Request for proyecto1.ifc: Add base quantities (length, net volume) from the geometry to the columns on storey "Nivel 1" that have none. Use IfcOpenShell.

First a look at what the model holds.

```python
import ifcopenshell
import ifcopenshell.util.element
import ifcopenshell.util.unit

model = ifcopenshell.open("proyecto1.ifc")
print(model.schema)
for unit_type in ("LENGTHUNIT", "AREAUNIT", "VOLUMEUNIT"):
    print(unit_type, ifcopenshell.util.unit.calculate_unit_scale(model, unit_type))
storey = next(s for s in model.by_type("IfcBuildingStorey") if s.Name == "Nivel 1")
columns = [e for e in ifcopenshell.util.element.get_decomposition(storey) if e.is_a("IfcColumn")]
for e in sorted(columns, key=lambda e: e.id()):
    print(e.id(), e.is_a(), e.Name, list(ifcopenshell.util.element.get_psets(e, qtos_only=True)), sep=" | ")
```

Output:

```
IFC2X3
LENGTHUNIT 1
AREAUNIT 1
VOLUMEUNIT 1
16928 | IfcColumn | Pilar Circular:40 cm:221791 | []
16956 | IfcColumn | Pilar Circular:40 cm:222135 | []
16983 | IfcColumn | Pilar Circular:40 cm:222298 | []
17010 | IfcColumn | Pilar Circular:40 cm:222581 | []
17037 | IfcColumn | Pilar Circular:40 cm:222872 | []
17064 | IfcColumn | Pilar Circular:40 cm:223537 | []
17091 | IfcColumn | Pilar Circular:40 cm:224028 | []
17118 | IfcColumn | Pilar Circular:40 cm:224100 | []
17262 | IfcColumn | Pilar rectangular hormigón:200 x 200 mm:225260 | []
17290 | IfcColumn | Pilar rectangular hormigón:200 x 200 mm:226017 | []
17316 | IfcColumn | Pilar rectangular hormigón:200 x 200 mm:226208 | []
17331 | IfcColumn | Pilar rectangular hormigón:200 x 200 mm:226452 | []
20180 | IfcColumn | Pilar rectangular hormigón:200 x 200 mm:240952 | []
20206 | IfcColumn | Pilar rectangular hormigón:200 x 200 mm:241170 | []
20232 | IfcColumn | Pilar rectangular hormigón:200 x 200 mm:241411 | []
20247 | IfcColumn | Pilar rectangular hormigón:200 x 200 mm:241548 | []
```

```python
import ifcopenshell
import ifcopenshell.api.pset
import ifcopenshell.geom
import ifcopenshell.util.element
import ifcopenshell.util.shape
import ifcopenshell.util.unit

model = ifcopenshell.open("proyecto1.ifc")
unit_scale = ifcopenshell.util.unit.calculate_unit_scale(model)
volume_scale = ifcopenshell.util.unit.calculate_unit_scale(model, "VOLUMEUNIT")
settings = ifcopenshell.geom.settings()

storey = next(s for s in model.by_type("IfcBuildingStorey") if s.Name == "Nivel 1")
columns = [e for e in ifcopenshell.util.element.get_decomposition(storey) if e.is_a("IfcColumn")]

for e in sorted(columns, key=lambda e: e.id()):
    if ifcopenshell.util.element.get_psets(e, qtos_only=True, should_inherit=False):
        continue
    # Geometry comes back in metres, in the element's own axes.
    shape = ifcopenshell.geom.create_shape(settings, e)
    values = {
        "Length": ifcopenshell.util.shape.get_z(shape.geometry) / unit_scale,
        "NetVolume": ifcopenshell.util.shape.get_volume(shape.geometry) / volume_scale,
    }
    qto = ifcopenshell.api.pset.add_qto(model, product=e, name="BaseQuantities")
    ifcopenshell.api.pset.edit_qto(model, qto=qto, properties=values)
    print(e.id(), {k: round(v, 3) for k, v in values.items()})

model.write("proyecto1_updated.ifc")
```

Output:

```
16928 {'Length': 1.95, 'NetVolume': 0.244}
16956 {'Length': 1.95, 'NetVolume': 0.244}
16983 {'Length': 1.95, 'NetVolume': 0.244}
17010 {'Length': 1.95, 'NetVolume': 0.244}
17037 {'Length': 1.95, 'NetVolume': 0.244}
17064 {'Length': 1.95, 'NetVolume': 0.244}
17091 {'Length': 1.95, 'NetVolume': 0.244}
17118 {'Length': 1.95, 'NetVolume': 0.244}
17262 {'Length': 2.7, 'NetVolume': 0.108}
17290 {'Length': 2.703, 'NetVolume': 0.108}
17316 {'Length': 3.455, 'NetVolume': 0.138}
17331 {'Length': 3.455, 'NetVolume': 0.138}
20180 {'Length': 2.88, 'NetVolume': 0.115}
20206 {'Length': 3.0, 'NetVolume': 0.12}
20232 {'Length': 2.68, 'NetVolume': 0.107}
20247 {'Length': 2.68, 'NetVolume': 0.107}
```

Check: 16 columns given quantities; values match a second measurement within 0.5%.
